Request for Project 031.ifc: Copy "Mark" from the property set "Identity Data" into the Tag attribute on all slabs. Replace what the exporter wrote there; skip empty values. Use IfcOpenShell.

First a look at what the model holds.

```python
import ifcopenshell
import ifcopenshell.util.element

model = ifcopenshell.open("Project 031.ifc")
print(model.schema)
slabs = model.by_type("IfcSlab")
print(len(slabs), "slabs")
for e in slabs[:8]:
    source = ifcopenshell.util.element.get_pset(e, "Identity Data", "Mark")
    target = e.Tag
    print(e.id(), repr(source), repr(target), sep=" | ")
```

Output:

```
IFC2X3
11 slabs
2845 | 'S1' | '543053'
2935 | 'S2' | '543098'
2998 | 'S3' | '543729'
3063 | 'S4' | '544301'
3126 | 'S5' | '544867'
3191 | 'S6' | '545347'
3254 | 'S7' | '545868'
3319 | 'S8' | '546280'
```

```python
import ifcopenshell
import ifcopenshell.util.element

model = ifcopenshell.open("Project 031.ifc")

count = 0
for e in model.by_type("IfcSlab"):
    value = ifcopenshell.util.element.get_pset(e, "Identity Data", "Mark")
    current = e.Tag
    if not value or not value.strip() or current == value:
        continue
    e.Tag = value
    count += 1

print(count, "slabs updated")

model.write("Project 031_updated.ifc")
```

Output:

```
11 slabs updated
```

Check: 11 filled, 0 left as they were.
